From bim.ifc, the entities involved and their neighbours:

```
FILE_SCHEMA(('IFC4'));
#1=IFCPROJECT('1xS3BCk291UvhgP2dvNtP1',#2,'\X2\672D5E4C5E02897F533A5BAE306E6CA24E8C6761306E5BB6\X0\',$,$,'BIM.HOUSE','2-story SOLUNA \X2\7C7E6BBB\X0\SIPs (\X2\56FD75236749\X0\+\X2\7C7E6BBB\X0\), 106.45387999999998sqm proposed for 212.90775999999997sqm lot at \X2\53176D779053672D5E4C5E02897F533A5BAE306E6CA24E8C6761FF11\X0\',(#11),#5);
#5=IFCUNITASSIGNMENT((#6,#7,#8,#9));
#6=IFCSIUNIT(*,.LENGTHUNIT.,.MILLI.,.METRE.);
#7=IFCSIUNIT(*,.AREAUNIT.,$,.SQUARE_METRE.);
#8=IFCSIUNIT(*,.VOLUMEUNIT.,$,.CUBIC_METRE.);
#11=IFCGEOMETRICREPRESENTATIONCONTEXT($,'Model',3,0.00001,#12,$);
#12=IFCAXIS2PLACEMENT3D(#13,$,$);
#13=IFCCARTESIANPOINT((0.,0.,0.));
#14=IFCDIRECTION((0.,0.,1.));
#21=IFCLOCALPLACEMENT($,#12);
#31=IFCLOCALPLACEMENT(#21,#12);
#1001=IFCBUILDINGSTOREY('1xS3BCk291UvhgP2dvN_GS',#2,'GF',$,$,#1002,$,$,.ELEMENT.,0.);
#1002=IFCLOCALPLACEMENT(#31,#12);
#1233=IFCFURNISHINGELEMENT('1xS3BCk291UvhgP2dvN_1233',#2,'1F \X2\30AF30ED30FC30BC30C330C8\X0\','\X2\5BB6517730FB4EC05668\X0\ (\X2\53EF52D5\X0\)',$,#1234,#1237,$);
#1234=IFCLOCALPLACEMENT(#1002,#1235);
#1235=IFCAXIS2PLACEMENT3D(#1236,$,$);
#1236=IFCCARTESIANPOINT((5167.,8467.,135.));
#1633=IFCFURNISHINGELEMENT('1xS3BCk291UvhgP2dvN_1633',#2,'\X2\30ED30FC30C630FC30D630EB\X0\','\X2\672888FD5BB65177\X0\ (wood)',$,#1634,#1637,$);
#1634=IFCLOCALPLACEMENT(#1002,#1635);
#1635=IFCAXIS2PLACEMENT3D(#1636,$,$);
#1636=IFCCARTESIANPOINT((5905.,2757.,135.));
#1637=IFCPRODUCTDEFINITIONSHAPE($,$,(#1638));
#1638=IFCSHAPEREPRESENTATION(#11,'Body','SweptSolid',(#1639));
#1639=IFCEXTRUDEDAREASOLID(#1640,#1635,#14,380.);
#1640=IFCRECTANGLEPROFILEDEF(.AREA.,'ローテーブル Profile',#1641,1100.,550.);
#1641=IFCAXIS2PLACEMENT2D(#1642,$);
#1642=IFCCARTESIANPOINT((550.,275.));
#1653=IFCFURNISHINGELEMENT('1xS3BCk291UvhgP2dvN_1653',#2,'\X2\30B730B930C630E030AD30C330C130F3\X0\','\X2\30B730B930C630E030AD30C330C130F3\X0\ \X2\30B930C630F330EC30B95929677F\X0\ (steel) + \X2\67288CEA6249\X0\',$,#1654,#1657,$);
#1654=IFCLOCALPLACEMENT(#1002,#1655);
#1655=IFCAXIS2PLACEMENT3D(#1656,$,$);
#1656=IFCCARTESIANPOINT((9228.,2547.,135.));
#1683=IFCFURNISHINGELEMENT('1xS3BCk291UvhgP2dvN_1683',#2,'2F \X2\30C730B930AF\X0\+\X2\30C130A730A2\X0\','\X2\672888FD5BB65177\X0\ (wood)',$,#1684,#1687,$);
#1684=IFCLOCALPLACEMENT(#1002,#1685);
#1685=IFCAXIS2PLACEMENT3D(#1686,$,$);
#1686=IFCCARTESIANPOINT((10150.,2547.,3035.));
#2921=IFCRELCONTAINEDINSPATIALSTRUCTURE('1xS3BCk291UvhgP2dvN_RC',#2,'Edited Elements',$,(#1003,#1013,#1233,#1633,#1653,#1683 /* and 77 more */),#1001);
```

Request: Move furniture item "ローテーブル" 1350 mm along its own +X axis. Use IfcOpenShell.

```python
import ifcopenshell
import ifcopenshell.api.geometry
import ifcopenshell.util.placement
import ifcopenshell.util.unit

model = ifcopenshell.open("bim.ifc")
unit_scale = ifcopenshell.util.unit.calculate_unit_scale(model)

item = model.by_guid("1xS3BCk291UvhgP2dvN_1633")
matrix = ifcopenshell.util.placement.get_local_placement(item.ObjectPlacement)
matrix[:3, 3] += matrix[:3, 0] * 1.35 / unit_scale
ifcopenshell.api.geometry.edit_object_placement(model, product=item, matrix=matrix, is_si=False)

print(ifcopenshell.util.placement.get_local_placement(item.ObjectPlacement).round(3) + 0.0)

model.write("bim_updated.ifc")
```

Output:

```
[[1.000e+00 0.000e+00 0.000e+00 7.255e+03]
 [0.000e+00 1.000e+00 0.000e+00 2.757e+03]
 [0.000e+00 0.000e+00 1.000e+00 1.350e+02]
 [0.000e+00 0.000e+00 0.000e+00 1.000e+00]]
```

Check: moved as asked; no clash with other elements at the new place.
